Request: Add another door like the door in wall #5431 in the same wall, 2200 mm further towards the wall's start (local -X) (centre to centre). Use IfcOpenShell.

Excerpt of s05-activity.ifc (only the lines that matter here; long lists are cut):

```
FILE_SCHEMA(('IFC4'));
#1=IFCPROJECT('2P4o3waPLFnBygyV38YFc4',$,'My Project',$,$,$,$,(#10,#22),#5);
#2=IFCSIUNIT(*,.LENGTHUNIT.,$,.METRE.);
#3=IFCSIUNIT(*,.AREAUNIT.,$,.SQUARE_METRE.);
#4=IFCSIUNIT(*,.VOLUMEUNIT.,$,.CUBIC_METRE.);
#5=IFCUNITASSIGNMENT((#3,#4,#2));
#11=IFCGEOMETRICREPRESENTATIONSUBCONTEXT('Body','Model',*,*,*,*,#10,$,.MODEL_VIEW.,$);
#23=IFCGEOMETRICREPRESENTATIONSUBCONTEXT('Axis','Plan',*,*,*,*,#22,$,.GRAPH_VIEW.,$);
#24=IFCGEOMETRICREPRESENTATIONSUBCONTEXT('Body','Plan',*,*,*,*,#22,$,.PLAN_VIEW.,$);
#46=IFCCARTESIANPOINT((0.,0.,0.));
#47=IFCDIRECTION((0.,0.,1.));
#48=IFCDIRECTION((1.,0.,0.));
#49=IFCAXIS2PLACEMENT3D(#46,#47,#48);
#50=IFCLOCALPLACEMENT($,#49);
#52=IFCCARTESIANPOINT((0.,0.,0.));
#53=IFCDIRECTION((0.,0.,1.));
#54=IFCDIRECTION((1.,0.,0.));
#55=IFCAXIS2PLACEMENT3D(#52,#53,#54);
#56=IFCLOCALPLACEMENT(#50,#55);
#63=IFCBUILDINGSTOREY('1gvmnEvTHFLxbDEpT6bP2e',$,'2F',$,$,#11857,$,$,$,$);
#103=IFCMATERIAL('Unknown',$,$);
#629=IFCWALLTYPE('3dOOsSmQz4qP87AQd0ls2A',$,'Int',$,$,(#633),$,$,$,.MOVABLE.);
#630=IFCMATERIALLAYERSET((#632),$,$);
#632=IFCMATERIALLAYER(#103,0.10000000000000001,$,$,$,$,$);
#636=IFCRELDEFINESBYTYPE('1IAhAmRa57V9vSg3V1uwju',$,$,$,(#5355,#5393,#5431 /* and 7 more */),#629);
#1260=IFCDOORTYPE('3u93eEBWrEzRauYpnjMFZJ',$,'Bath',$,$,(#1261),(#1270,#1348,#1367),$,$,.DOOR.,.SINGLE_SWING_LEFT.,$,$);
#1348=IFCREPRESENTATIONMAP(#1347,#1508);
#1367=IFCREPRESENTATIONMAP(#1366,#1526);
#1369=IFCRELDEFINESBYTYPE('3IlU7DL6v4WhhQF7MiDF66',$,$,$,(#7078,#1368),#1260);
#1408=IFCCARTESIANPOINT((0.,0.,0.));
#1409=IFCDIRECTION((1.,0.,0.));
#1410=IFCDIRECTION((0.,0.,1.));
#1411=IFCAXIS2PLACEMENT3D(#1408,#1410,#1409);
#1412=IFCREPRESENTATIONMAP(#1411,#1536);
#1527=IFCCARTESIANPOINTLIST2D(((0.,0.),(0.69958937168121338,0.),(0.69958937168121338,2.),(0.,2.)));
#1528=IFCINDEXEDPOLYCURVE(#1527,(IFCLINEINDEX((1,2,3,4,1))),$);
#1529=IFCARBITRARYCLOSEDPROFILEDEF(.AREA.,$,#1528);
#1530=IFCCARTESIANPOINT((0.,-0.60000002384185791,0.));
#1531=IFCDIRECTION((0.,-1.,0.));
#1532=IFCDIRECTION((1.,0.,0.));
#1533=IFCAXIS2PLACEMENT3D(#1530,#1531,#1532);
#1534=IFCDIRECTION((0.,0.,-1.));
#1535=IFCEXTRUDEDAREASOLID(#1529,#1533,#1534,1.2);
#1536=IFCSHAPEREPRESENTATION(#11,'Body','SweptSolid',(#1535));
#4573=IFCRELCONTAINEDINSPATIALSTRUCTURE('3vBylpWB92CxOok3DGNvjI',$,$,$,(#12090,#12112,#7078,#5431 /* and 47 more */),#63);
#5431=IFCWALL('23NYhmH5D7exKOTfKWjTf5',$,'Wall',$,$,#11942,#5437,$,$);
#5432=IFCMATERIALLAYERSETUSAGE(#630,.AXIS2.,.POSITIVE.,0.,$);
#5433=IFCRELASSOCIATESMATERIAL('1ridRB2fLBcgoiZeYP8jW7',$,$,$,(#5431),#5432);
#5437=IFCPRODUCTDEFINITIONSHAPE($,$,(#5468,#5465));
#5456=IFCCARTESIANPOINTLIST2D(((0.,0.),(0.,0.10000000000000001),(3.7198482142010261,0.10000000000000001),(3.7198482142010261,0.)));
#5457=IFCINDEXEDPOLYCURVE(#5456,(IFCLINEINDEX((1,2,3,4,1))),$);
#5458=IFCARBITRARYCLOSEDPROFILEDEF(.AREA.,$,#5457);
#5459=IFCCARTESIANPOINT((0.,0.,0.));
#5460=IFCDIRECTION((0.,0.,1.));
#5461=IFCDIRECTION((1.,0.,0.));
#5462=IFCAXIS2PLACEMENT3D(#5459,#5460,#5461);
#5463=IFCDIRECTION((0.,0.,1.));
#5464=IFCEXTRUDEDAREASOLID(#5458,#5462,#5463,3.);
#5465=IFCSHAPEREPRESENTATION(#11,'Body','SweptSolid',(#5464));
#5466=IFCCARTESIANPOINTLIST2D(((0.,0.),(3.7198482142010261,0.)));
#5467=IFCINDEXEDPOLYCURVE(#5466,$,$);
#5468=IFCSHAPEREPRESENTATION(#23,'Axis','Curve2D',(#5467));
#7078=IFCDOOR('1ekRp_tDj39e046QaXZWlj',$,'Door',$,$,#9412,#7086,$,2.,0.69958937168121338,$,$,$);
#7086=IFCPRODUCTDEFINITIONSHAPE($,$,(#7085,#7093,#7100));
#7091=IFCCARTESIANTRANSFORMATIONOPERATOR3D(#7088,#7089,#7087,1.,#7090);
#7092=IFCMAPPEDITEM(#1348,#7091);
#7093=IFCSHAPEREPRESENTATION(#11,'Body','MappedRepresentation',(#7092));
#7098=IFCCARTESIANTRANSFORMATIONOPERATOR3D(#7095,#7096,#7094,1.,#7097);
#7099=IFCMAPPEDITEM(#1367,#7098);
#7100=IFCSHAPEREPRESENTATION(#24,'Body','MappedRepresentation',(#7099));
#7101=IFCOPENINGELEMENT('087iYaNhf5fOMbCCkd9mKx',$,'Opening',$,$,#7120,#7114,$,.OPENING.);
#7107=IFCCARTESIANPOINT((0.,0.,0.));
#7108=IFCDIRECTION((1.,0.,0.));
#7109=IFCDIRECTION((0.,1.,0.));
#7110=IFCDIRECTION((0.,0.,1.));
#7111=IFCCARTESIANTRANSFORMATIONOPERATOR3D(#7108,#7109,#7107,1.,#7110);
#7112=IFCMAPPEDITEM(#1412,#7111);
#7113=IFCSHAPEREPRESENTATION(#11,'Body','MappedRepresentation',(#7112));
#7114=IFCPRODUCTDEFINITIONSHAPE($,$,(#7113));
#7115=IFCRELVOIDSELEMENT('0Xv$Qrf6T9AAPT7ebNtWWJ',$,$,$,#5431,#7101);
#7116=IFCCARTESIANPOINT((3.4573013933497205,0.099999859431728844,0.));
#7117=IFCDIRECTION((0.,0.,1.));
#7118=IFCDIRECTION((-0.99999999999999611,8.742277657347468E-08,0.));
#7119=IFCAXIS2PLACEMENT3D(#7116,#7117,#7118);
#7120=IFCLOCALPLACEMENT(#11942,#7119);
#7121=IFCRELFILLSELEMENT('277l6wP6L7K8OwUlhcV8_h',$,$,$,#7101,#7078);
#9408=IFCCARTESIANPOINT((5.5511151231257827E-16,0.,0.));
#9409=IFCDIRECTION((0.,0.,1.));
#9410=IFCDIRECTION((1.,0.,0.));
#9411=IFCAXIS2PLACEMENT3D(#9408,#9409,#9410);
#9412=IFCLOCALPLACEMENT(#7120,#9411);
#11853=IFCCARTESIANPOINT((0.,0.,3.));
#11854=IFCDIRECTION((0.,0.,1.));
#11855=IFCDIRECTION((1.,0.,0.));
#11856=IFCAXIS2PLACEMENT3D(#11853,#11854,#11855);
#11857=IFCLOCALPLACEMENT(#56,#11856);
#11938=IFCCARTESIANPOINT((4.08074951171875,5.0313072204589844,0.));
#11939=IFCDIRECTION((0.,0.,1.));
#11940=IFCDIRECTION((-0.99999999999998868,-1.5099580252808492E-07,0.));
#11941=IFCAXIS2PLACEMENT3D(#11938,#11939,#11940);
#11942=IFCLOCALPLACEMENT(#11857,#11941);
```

```python
import ifcopenshell
import ifcopenshell.api.feature
import ifcopenshell.api.geometry
import ifcopenshell.api.root
import ifcopenshell.geom
import ifcopenshell.util.element
import ifcopenshell.util.placement
import ifcopenshell.util.shape
import ifcopenshell.util.unit

model = ifcopenshell.open("s05-activity.ifc")
unit_scale = ifcopenshell.util.unit.calculate_unit_scale(model)
settings = ifcopenshell.geom.settings()


def volume(element):
    """Net volume in cubic metres, openings subtracted."""
    shape = ifcopenshell.geom.create_shape(settings, element)
    return ifcopenshell.util.shape.get_volume(shape.geometry)


door = model.by_guid("1ekRp_tDj39e046QaXZWlj")
opening = door.FillsVoids[0].RelatingOpeningElement
wall = opening.VoidsElements[0].RelatingBuildingElement
before = volume(wall)
shift = ifcopenshell.util.placement.get_local_placement(wall.ObjectPlacement)[:3, 0] * -2.2 / unit_scale

# copy_class copies the void relationship, type, container and properties, but no geometry.
new_opening = ifcopenshell.api.root.copy_class(model, product=opening)
new_opening.Representation = ifcopenshell.util.element.copy_deep(
    model, opening.Representation, exclude=["IfcGeometricRepresentationContext", "IfcRepresentationMap"]
)
new_door = ifcopenshell.api.root.copy_class(model, product=door)
new_door.Representation = ifcopenshell.util.element.copy_deep(
    model, door.Representation, exclude=["IfcGeometricRepresentationContext", "IfcRepresentationMap"]
)
ifcopenshell.api.feature.add_filling(model, opening=new_opening, element=new_door)

for old, new in ((opening, new_opening), (door, new_door)):
    matrix = ifcopenshell.util.placement.get_local_placement(old.ObjectPlacement)
    matrix[:3, 3] += shift
    ifcopenshell.api.geometry.edit_object_placement(model, product=new, matrix=matrix, is_si=False)

after = volume(wall)

print(f"wall volume {before:.3f} -> {after:.3f} m3")

model.write("s05-activity_rev.ifc")
```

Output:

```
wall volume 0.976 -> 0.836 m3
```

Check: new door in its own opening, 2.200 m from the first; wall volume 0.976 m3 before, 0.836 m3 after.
